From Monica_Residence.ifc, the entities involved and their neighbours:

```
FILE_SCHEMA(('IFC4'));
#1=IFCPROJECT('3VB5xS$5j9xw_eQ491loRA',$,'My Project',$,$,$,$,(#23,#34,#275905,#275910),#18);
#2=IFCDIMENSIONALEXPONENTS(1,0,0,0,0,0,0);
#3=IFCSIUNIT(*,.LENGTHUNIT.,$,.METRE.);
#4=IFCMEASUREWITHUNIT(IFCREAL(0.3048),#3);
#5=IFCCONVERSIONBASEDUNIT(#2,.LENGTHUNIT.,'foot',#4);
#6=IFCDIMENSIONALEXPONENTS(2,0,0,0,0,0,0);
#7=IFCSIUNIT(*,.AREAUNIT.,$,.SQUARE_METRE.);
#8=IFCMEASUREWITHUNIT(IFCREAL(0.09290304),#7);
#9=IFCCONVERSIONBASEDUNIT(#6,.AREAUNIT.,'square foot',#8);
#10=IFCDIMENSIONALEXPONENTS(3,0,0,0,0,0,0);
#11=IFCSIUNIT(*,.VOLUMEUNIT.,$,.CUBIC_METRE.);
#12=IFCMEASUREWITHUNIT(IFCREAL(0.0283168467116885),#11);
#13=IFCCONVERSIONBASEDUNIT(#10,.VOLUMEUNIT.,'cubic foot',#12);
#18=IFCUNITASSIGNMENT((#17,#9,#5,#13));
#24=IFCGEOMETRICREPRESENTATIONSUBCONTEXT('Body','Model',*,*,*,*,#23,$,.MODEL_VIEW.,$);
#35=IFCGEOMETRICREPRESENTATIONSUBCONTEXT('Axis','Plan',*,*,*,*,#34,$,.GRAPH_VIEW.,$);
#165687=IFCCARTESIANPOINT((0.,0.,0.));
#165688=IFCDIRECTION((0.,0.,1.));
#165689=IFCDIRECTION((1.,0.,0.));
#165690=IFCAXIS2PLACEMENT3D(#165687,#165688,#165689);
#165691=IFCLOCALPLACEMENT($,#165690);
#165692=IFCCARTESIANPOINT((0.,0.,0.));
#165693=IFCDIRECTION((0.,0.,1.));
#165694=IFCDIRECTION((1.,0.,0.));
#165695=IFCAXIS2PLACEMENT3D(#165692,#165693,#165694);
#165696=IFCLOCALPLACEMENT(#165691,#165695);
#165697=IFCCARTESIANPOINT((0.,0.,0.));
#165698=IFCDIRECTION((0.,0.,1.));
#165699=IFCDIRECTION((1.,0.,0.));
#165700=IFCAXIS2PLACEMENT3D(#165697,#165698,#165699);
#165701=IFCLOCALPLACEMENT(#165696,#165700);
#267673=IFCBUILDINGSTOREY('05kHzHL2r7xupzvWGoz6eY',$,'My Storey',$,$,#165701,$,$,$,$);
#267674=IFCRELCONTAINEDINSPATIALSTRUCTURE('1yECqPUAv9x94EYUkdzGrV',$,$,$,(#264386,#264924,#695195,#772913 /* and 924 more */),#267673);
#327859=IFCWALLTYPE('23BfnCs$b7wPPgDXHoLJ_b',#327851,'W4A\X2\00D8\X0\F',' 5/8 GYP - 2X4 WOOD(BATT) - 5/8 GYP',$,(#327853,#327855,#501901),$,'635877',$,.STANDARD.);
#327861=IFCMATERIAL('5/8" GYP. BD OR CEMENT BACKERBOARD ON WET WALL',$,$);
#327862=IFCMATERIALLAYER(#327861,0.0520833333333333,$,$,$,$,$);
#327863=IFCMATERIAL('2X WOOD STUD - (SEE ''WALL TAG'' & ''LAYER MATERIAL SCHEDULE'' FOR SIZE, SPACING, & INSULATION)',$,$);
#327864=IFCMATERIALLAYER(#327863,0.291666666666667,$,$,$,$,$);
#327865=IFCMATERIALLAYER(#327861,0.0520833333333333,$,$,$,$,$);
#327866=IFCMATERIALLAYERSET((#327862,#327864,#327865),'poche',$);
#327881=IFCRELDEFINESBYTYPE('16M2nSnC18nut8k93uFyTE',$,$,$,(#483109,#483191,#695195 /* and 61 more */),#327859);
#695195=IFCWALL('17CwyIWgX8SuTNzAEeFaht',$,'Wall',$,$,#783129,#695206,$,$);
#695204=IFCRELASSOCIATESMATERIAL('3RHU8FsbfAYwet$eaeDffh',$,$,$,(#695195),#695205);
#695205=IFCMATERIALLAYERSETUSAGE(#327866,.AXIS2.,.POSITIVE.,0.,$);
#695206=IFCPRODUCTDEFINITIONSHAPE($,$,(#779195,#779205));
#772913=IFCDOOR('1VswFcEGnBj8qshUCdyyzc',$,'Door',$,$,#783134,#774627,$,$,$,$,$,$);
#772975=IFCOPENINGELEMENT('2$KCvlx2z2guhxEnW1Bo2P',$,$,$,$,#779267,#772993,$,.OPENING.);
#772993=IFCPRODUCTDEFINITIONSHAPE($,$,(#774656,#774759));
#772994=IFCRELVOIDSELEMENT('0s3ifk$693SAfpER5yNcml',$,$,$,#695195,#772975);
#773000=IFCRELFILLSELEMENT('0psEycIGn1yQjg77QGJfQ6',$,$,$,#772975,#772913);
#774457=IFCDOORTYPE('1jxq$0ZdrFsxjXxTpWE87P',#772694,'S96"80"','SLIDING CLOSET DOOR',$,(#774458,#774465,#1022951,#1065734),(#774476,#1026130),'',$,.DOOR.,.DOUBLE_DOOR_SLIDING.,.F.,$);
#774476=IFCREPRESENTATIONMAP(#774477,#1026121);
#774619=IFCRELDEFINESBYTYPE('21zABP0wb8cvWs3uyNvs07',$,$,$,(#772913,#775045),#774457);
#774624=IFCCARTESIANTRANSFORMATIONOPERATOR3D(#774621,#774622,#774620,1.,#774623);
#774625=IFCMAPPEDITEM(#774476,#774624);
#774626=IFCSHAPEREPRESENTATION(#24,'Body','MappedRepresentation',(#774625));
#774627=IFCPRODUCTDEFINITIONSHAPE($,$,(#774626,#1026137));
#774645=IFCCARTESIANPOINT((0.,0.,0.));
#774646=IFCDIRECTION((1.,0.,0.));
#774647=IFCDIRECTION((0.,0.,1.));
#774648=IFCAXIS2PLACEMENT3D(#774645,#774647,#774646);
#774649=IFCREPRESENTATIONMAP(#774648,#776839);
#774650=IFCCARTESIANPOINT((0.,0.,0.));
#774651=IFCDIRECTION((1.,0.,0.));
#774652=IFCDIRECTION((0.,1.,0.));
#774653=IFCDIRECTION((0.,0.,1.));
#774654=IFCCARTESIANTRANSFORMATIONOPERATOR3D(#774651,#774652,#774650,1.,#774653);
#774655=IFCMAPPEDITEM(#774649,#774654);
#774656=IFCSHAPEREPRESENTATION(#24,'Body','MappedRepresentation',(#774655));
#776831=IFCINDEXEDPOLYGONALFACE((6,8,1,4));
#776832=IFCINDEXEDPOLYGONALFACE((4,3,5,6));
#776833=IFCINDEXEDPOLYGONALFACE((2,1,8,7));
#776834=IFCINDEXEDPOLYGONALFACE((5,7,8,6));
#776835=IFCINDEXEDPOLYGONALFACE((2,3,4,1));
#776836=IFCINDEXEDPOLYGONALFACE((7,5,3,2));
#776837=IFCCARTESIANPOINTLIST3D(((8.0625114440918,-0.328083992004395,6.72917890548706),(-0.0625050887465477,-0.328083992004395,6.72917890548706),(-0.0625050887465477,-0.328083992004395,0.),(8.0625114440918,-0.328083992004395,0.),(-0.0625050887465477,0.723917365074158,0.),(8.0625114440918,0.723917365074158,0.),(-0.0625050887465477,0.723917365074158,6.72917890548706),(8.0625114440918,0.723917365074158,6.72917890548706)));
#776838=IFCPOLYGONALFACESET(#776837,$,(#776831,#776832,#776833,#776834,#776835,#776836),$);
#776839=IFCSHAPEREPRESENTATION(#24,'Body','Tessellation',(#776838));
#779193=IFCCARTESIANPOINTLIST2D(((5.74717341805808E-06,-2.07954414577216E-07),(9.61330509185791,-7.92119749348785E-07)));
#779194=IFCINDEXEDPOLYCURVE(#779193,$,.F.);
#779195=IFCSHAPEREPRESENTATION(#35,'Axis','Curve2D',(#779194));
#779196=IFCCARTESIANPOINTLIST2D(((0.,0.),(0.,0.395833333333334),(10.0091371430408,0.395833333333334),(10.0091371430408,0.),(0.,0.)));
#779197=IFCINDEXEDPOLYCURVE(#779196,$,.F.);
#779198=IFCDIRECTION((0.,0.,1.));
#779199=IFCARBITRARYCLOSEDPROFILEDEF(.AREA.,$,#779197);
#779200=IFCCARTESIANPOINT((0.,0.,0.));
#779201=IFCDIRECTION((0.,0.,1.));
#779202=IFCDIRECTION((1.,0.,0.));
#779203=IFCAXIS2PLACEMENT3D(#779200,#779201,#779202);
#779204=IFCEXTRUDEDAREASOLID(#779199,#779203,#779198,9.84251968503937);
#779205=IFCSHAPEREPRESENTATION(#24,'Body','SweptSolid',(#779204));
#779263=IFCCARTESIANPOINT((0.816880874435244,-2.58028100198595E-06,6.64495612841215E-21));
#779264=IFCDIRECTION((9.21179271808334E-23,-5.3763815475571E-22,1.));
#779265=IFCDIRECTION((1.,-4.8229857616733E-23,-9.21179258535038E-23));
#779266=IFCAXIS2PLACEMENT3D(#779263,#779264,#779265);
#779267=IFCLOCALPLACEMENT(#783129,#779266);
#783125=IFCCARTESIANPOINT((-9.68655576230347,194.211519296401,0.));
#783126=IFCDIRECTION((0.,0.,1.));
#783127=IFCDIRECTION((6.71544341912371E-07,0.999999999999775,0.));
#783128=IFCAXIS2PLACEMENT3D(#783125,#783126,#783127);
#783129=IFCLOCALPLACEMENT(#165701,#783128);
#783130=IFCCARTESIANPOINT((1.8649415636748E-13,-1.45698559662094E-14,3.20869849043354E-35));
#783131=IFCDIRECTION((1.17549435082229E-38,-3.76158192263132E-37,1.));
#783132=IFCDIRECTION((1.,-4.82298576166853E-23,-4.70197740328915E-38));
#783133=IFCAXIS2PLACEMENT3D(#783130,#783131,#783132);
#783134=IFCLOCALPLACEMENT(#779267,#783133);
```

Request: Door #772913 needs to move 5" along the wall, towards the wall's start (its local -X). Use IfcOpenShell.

```python
import ifcopenshell
import ifcopenshell.api.geometry
import ifcopenshell.util.placement
import ifcopenshell.util.unit

model = ifcopenshell.open("Monica_Residence.ifc")
unit_scale = ifcopenshell.util.unit.calculate_unit_scale(model)

door = model.by_guid("1VswFcEGnBj8qshUCdyyzc")
opening = door.FillsVoids[0].RelatingOpeningElement
wall = opening.VoidsElements[0].RelatingBuildingElement

wall_matrix = ifcopenshell.util.placement.get_local_placement(wall.ObjectPlacement)
shift = wall_matrix[:3, 0] * -5 * 0.0254 / unit_scale
before = ifcopenshell.util.placement.get_local_placement(door.ObjectPlacement)[:3, 3].copy()

# The door is placed relative to its opening, so it follows when the opening moves.
matrix = ifcopenshell.util.placement.get_local_placement(opening.ObjectPlacement)
matrix[:3, 3] += shift
ifcopenshell.api.geometry.edit_object_placement(
    model, product=opening, matrix=matrix, is_si=False, should_transform_children=True
)

after = ifcopenshell.util.placement.get_local_placement(door.ObjectPlacement)[:3, 3]
print("door moved by", (after - before).round(3) + 0.0)

model.write("Monica_Residence_rev.ifc")
```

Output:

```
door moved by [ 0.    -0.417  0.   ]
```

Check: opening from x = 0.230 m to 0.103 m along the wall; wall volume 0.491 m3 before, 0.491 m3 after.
